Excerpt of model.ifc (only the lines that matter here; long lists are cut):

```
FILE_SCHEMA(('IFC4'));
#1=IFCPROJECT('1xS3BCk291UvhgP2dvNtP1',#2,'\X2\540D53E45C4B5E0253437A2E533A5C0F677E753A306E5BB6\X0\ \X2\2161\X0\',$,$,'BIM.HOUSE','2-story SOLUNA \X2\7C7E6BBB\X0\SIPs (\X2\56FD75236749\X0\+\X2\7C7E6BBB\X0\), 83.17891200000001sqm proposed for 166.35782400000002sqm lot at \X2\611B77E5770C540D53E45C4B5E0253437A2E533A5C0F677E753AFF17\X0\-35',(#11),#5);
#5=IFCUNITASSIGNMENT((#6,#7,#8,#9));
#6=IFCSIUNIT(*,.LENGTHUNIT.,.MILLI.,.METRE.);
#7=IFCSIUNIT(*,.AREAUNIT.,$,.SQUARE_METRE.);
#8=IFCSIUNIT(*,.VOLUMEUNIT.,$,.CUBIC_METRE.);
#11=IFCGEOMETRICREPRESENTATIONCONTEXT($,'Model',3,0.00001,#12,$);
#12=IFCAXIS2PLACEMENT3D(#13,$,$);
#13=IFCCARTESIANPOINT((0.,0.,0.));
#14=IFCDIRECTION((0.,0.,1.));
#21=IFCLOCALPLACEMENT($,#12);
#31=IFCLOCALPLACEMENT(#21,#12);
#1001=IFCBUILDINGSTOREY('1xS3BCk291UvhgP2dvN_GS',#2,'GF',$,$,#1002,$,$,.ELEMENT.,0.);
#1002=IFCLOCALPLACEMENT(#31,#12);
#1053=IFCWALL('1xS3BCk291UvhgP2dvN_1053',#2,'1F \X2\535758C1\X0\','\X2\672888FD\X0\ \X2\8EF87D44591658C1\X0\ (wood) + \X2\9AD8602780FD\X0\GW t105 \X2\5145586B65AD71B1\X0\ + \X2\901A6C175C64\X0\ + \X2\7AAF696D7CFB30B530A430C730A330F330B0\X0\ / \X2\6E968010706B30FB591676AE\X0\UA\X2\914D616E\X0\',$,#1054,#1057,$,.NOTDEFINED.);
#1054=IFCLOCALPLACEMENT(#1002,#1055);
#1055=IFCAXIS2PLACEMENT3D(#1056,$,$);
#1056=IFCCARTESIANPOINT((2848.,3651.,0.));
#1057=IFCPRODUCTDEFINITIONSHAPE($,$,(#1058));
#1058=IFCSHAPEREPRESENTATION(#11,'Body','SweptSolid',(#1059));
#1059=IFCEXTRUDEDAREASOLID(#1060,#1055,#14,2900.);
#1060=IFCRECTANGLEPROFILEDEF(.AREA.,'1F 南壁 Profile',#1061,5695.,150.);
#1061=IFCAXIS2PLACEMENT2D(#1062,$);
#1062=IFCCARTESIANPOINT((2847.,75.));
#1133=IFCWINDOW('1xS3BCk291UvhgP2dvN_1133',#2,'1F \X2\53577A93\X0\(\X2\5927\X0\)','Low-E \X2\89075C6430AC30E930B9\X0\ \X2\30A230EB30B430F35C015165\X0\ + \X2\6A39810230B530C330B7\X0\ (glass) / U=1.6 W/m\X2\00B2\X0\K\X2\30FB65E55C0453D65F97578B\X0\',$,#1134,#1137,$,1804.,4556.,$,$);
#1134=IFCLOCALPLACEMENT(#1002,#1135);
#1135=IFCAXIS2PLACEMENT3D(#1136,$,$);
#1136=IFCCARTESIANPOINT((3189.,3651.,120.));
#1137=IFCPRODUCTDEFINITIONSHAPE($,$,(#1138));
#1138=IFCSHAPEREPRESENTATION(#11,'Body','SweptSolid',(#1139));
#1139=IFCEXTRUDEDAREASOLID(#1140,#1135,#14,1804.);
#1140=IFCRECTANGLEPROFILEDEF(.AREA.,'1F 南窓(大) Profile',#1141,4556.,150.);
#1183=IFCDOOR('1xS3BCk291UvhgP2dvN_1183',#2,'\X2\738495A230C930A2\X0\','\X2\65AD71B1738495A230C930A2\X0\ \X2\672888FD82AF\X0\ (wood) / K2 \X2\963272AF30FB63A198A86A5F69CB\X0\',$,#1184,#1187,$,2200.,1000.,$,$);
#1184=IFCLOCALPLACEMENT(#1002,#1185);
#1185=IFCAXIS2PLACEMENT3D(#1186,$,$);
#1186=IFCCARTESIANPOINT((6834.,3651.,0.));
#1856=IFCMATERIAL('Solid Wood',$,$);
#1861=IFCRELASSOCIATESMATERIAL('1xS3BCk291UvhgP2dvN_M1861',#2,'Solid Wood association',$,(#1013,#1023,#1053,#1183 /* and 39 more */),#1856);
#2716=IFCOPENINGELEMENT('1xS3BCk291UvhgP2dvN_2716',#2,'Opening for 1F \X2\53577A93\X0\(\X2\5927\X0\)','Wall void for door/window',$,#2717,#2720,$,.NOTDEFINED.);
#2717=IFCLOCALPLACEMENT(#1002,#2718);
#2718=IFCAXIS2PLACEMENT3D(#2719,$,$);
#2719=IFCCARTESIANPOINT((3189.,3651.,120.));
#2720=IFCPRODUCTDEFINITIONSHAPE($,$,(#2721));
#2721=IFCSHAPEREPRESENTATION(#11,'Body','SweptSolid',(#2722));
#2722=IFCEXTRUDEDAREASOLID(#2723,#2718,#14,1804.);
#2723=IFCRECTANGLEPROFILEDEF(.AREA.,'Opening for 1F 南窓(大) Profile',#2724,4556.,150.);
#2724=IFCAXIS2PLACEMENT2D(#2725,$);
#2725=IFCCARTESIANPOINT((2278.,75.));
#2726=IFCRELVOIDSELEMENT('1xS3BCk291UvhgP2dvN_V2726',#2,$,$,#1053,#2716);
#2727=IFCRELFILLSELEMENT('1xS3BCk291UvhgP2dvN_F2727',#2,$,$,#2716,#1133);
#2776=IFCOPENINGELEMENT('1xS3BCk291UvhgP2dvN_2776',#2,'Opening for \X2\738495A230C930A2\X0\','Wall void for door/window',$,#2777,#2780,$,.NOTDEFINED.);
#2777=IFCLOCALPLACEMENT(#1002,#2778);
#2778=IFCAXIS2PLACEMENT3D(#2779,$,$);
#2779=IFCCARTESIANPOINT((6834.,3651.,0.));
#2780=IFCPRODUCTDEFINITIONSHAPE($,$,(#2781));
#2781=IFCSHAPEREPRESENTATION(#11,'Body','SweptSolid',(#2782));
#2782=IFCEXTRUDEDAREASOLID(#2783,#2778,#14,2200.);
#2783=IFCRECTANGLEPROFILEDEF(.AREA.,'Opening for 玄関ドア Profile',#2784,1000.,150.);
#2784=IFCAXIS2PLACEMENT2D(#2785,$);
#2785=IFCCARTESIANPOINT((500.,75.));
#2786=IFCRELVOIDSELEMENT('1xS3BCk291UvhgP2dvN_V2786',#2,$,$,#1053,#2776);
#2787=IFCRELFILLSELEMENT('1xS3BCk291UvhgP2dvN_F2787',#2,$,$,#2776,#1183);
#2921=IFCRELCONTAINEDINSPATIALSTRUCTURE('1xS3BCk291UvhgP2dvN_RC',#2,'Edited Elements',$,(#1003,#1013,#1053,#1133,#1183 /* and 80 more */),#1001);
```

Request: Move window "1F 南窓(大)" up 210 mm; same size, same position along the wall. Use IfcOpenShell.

```python
import numpy as np
import ifcopenshell
import ifcopenshell.api.geometry
import ifcopenshell.util.placement
import ifcopenshell.util.unit

model = ifcopenshell.open("model.ifc")
unit_scale = ifcopenshell.util.unit.calculate_unit_scale(model)

window = model.by_id(1133)
opening = window.FillsVoids[0].RelatingOpeningElement
dz = 0.21 / unit_scale

shift = np.array([0.0, 0.0, dz])
# The window is not placed relative to its opening, so move both.
for product in (opening, window):
    matrix = ifcopenshell.util.placement.get_local_placement(product.ObjectPlacement)
    matrix[:3, 3] += shift
    ifcopenshell.api.geometry.edit_object_placement(model, product=product, matrix=matrix, is_si=False)

print(f"moved by {dz * unit_scale:+.3f} m")

model.write("model_v2.ifc")
```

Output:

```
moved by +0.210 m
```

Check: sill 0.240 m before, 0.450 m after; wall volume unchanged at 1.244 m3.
